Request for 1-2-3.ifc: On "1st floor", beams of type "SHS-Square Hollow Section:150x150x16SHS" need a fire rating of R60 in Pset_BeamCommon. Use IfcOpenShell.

First a look at what the model holds.

```python
import ifcopenshell
import ifcopenshell.util.element

model = ifcopenshell.open("1-2-3.ifc")
print(model.schema)
storey = next(s for s in model.by_type("IfcBuildingStorey") if s.Name == "1st floor")
beams = [e for e in ifcopenshell.util.element.get_decomposition(storey) if e.is_a("IfcBeam")]
seen = {}
for e in beams:
    element_type = ifcopenshell.util.element.get_type(e)
    key = (element_type.Name if element_type != e and element_type else None, ifcopenshell.util.element.get_pset(e, "Pset_BeamCommon", "FireRating"))
    seen[key] = seen.get(key, 0) + 1
for (name, value), count in sorted(seen.items(), key=str):
    print(count, "x", name, "|", value)
```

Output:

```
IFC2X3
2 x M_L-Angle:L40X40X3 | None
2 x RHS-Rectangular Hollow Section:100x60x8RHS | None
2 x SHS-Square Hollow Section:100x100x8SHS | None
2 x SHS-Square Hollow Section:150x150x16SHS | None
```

```python
import ifcopenshell
import ifcopenshell.api.pset
import ifcopenshell.util.element

model = ifcopenshell.open("1-2-3.ifc")

storey = next(s for s in model.by_type("IfcBuildingStorey") if s.Name == "1st floor")
beams = [e for e in ifcopenshell.util.element.get_decomposition(storey) if e.is_a("IfcBeam")]

count = 0
for e in beams:
    element_type = ifcopenshell.util.element.get_type(e)
    if element_type in (None, e) or element_type.Name != "SHS-Square Hollow Section:150x150x16SHS":
        continue
    # add_pset returns the element's existing set when there is one.
    pset = ifcopenshell.api.pset.add_pset(model, product=e, name="Pset_BeamCommon")
    ifcopenshell.api.pset.edit_pset(model, pset=pset, properties={"FireRating": "R60"})
    count += 1

print(count, "beams updated")

model.write("1-2-3_rev.ifc")
```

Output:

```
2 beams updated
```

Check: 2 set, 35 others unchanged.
